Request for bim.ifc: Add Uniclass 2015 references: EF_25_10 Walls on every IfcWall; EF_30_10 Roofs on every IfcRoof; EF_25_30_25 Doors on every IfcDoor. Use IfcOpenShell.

First a look at what the model holds.

```python
import ifcopenshell

model = ifcopenshell.open("bim.ifc")
print(model.schema)
print("classifications:", [c.Name for c in model.by_type("IfcClassification")])
for ifc_class in ("IfcDoor", "IfcRoof", "IfcStair", "IfcWall", "IfcWindow"):
    print(ifc_class, len(model.by_type(ifc_class)))
```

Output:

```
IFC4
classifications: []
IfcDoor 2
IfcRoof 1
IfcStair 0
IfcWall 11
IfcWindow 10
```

```python
import ifcopenshell
import ifcopenshell.api.classification

model = ifcopenshell.open("bim.ifc")

system = ifcopenshell.api.classification.add_classification(model, classification="Uniclass 2015")

codes = {
    "IfcWall": ("EF_25_10", "Walls"),
    "IfcRoof": ("EF_30_10", "Roofs"),
    "IfcDoor": ("EF_25_30_25", "Doors"),
}
for ifc_class, (code, name) in codes.items():
    products = model.by_type(ifc_class)
    ifcopenshell.api.classification.add_reference(
        model, products=products, classification=system, identification=code, name=name
    )
    print(code, len(products))

model.write("bim-out.ifc")
```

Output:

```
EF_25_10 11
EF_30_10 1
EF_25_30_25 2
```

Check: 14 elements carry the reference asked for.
